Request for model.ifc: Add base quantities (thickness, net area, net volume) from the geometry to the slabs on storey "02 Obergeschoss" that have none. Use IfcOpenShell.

First a look at what the model holds.

```python
import ifcopenshell
import ifcopenshell.util.element
import ifcopenshell.util.unit

model = ifcopenshell.open("model.ifc")
print(model.schema)
for unit_type in ("LENGTHUNIT", "AREAUNIT", "VOLUMEUNIT"):
    print(unit_type, ifcopenshell.util.unit.calculate_unit_scale(model, unit_type))
storey = next(s for s in model.by_type("IfcBuildingStorey") if s.Name == "02 Obergeschoss")
slabs = [e for e in ifcopenshell.util.element.get_decomposition(storey) if e.is_a("IfcSlab")]
for e in sorted(slabs, key=lambda e: e.id()):
    print(e.id(), e.is_a(), e.Name, list(ifcopenshell.util.element.get_psets(e, qtos_only=True)), sep=" | ")
```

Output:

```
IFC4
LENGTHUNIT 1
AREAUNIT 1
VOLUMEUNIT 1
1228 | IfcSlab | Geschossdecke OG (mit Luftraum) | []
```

```python
import ifcopenshell
import ifcopenshell.api.pset
import ifcopenshell.geom
import ifcopenshell.util.element
import ifcopenshell.util.shape
import ifcopenshell.util.unit

model = ifcopenshell.open("model.ifc")
unit_scale = ifcopenshell.util.unit.calculate_unit_scale(model)
area_scale = ifcopenshell.util.unit.calculate_unit_scale(model, "AREAUNIT")
volume_scale = ifcopenshell.util.unit.calculate_unit_scale(model, "VOLUMEUNIT")
settings = ifcopenshell.geom.settings()

storey = next(s for s in model.by_type("IfcBuildingStorey") if s.Name == "02 Obergeschoss")
slabs = [e for e in ifcopenshell.util.element.get_decomposition(storey) if e.is_a("IfcSlab")]

for e in sorted(slabs, key=lambda e: e.id()):
    if ifcopenshell.util.element.get_psets(e, qtos_only=True, should_inherit=False):
        continue
    # Geometry comes back in metres, in the element's own axes.
    shape = ifcopenshell.geom.create_shape(settings, e)
    values = {
        "Width": ifcopenshell.util.shape.get_z(shape.geometry) / unit_scale,
        "NetArea": ifcopenshell.util.shape.get_footprint_area(shape.geometry) / area_scale,
        "NetVolume": ifcopenshell.util.shape.get_volume(shape.geometry) / volume_scale,
    }
    qto = ifcopenshell.api.pset.add_qto(model, product=e, name="Qto_SlabBaseQuantities")
    ifcopenshell.api.pset.edit_qto(model, qto=qto, properties=values)
    print(e.id(), {k: round(v, 3) for k, v in values.items()})

model.write("model_v2.ifc")
```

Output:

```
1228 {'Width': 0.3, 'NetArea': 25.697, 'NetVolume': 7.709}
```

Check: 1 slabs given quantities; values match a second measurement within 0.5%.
